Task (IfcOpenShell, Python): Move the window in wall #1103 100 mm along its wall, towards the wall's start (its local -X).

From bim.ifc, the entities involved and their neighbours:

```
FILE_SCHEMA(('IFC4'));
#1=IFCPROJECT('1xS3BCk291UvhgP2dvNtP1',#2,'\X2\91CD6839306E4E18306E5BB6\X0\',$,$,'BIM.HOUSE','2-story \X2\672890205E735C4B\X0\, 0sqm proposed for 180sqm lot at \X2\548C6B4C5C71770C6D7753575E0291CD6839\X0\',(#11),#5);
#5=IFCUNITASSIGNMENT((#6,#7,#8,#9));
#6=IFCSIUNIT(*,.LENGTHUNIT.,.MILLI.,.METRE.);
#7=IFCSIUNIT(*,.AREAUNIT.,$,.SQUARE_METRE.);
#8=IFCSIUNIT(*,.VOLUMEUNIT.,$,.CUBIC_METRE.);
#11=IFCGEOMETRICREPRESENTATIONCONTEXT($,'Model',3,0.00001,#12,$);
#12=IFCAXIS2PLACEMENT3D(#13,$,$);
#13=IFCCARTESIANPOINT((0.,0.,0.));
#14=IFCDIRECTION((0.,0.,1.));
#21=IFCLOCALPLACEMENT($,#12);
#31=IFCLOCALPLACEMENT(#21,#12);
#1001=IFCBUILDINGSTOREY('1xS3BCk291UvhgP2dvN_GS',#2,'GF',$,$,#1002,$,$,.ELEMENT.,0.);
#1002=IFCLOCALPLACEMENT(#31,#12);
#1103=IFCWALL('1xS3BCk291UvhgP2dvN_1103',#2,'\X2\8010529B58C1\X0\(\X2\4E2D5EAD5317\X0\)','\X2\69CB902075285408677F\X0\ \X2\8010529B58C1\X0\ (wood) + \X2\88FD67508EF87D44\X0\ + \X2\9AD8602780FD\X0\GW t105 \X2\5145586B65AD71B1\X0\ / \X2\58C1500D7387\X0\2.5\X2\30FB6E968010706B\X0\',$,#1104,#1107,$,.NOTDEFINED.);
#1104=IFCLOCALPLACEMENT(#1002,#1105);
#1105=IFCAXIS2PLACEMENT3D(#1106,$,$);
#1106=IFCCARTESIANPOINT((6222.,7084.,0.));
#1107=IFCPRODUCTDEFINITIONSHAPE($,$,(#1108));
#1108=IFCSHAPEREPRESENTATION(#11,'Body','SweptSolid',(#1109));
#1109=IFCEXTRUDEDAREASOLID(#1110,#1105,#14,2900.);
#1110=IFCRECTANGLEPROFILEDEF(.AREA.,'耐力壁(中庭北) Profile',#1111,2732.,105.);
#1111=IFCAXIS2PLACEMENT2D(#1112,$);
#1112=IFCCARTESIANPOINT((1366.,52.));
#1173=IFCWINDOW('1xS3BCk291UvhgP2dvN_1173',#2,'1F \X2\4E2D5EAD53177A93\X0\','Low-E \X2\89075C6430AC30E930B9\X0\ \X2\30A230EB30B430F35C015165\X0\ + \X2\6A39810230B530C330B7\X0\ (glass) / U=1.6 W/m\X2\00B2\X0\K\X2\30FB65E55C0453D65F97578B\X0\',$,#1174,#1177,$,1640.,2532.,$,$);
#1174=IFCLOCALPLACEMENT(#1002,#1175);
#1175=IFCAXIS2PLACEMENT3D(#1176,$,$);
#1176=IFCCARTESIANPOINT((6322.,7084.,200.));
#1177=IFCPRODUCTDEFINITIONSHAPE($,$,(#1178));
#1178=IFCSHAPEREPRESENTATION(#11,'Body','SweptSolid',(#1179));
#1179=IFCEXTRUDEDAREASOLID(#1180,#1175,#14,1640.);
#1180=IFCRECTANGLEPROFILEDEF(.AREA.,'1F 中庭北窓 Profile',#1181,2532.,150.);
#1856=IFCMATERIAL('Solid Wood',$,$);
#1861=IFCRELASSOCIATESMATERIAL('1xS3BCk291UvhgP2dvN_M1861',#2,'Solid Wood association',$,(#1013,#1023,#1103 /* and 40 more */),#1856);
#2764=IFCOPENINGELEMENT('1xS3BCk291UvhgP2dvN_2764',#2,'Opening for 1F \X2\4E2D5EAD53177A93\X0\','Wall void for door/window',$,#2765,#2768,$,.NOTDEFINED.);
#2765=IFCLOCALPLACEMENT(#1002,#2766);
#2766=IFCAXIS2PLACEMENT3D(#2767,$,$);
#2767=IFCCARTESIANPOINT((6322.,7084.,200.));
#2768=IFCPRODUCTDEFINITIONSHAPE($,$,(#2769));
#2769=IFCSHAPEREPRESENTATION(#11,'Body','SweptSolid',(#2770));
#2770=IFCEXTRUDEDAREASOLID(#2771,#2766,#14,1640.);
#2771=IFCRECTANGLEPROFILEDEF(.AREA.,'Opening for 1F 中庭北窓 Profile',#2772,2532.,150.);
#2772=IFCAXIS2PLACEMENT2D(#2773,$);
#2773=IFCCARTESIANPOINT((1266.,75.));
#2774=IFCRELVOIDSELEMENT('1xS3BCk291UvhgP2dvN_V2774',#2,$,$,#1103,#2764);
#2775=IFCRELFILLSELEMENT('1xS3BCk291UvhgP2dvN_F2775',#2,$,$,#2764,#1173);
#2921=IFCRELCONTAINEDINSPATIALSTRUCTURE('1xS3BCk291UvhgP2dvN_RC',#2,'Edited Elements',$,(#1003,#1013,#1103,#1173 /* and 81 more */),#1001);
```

```python
import ifcopenshell
import ifcopenshell.api.geometry
import ifcopenshell.util.placement

model = ifcopenshell.open("bim.ifc")

window = model.by_guid("1xS3BCk291UvhgP2dvN_1173")
opening = window.FillsVoids[0].RelatingOpeningElement
wall = opening.VoidsElements[0].RelatingBuildingElement

wall_matrix = ifcopenshell.util.placement.get_local_placement(wall.ObjectPlacement)
shift = wall_matrix[:3, 0] * -100.0
before = ifcopenshell.util.placement.get_local_placement(window.ObjectPlacement)[:3, 3].copy()

# The window is not placed relative to its opening, so move both.
for product in (opening, window):
    matrix = ifcopenshell.util.placement.get_local_placement(product.ObjectPlacement)
    matrix[:3, 3] += shift
    ifcopenshell.api.geometry.edit_object_placement(model, product=product, matrix=matrix, is_si=False)

after = ifcopenshell.util.placement.get_local_placement(window.ObjectPlacement)[:3, 3]
print("window moved by", (after - before).round(3) + 0.0)

model.write("bim_v2.ifc")
```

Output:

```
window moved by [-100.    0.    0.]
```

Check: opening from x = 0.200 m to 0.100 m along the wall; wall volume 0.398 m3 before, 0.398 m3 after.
